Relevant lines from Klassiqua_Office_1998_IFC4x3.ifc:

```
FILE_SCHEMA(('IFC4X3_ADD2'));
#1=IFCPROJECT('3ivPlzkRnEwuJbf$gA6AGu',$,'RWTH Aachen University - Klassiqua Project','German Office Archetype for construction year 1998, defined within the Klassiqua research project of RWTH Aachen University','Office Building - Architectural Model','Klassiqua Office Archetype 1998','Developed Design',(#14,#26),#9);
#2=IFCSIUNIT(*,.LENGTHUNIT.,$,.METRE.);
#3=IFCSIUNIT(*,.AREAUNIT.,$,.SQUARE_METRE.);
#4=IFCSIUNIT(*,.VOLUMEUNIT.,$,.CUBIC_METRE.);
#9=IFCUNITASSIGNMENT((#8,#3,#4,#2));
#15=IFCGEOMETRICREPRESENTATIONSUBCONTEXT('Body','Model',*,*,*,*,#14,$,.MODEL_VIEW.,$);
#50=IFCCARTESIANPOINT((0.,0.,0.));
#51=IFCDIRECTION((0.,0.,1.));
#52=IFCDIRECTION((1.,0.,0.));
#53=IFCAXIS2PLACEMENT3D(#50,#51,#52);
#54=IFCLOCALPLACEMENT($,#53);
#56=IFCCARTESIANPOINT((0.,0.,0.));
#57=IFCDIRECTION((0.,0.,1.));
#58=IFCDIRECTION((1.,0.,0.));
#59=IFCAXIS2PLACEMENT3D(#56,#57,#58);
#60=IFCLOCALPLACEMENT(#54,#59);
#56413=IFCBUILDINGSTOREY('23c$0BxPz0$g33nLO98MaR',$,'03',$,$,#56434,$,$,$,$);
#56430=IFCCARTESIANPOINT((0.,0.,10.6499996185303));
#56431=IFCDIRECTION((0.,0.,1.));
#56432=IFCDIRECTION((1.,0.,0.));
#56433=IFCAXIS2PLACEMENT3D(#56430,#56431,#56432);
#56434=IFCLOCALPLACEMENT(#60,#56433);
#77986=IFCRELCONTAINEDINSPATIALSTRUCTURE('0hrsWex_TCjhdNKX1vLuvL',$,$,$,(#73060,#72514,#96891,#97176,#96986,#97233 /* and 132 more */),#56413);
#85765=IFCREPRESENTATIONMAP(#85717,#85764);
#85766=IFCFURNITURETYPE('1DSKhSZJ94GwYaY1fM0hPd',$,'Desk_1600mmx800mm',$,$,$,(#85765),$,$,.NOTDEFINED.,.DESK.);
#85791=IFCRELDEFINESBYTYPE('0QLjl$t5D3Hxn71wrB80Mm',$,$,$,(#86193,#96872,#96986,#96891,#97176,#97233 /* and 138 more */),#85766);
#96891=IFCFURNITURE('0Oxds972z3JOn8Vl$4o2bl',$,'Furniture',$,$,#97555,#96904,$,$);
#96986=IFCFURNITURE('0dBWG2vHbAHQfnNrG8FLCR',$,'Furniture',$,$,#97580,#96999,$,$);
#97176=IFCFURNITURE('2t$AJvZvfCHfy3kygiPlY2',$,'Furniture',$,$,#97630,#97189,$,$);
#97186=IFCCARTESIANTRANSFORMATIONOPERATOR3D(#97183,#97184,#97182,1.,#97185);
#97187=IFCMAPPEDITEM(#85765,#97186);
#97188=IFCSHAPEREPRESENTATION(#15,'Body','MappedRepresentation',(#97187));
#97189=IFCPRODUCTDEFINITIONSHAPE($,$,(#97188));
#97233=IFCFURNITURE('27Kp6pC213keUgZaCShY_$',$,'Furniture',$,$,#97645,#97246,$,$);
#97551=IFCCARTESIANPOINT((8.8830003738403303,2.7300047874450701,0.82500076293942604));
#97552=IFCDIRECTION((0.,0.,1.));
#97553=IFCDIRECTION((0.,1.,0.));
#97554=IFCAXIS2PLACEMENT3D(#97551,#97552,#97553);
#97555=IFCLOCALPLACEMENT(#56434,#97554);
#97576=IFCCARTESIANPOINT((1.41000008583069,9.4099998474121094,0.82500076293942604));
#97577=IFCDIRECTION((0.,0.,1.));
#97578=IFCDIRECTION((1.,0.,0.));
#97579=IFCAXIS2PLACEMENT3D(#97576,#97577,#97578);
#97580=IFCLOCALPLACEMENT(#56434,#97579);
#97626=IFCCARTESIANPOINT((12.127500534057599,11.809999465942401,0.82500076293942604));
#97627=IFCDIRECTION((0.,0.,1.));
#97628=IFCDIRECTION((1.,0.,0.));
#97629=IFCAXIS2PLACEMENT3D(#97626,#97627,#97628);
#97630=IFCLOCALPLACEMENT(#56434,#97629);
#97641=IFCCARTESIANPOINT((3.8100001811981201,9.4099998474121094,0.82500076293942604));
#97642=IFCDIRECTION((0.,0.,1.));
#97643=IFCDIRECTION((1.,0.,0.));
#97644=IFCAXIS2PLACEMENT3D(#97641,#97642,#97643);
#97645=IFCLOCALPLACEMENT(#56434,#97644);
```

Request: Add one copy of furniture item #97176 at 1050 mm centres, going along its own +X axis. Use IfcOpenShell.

```python
import ifcopenshell
import ifcopenshell.api.geometry
import ifcopenshell.api.root
import ifcopenshell.util.element
import ifcopenshell.util.placement
import ifcopenshell.util.unit

model = ifcopenshell.open("Klassiqua_Office_1998_IFC4x3.ifc")
unit_scale = ifcopenshell.util.unit.calculate_unit_scale(model)

source = model.by_guid("2t$AJvZvfCHfy3kygiPlY2")
base = ifcopenshell.util.placement.get_local_placement(source.ObjectPlacement)
step = base[:3, 0] * 1.05 / unit_scale

for i in range(1, 2):
    copy = ifcopenshell.api.root.copy_class(model, product=source)
    copy.Representation = ifcopenshell.util.element.copy_deep(
        model, source.Representation, exclude=["IfcGeometricRepresentationContext", "IfcRepresentationMap"]
    )
    matrix = base.copy()
    matrix[:3, 3] += i * step
    print("added at", matrix[:3, 3].round(3) + 0.0)
    ifcopenshell.api.geometry.edit_object_placement(model, product=copy, matrix=matrix, is_si=False)

model.write("Klassiqua_Office_1998_IFC4x3_rev.ifc")
```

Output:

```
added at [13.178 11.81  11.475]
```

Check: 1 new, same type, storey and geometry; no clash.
